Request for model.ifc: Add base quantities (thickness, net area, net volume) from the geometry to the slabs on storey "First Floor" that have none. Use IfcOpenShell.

First a look at what the model holds.

```python
import ifcopenshell
import ifcopenshell.util.element
import ifcopenshell.util.unit

model = ifcopenshell.open("model.ifc")
print(model.schema)
for unit_type in ("LENGTHUNIT", "AREAUNIT", "VOLUMEUNIT"):
    print(unit_type, ifcopenshell.util.unit.calculate_unit_scale(model, unit_type))
storey = next(s for s in model.by_type("IfcBuildingStorey") if s.Name == "First Floor")
slabs = [e for e in ifcopenshell.util.element.get_decomposition(storey) if e.is_a("IfcSlab")]
for e in sorted(slabs, key=lambda e: e.id()):
    print(e.id(), e.is_a(), e.Name, list(ifcopenshell.util.element.get_psets(e, qtos_only=True)), sep=" | ")
```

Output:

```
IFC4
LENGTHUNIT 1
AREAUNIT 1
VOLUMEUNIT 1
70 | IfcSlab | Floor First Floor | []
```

```python
import ifcopenshell
import ifcopenshell.api.pset
import ifcopenshell.geom
import ifcopenshell.util.element
import ifcopenshell.util.shape
import ifcopenshell.util.unit

model = ifcopenshell.open("model.ifc")
unit_scale = ifcopenshell.util.unit.calculate_unit_scale(model)
area_scale = ifcopenshell.util.unit.calculate_unit_scale(model, "AREAUNIT")
volume_scale = ifcopenshell.util.unit.calculate_unit_scale(model, "VOLUMEUNIT")
settings = ifcopenshell.geom.settings()

storey = next(s for s in model.by_type("IfcBuildingStorey") if s.Name == "First Floor")
slabs = [e for e in ifcopenshell.util.element.get_decomposition(storey) if e.is_a("IfcSlab")]

for e in sorted(slabs, key=lambda e: e.id()):
    if ifcopenshell.util.element.get_psets(e, qtos_only=True, should_inherit=False):
        continue
    # Geometry comes back in metres, in the element's own axes.
    shape = ifcopenshell.geom.create_shape(settings, e)
    values = {
        "Width": ifcopenshell.util.shape.get_z(shape.geometry) / unit_scale,
        "NetArea": ifcopenshell.util.shape.get_footprint_area(shape.geometry) / area_scale,
        "NetVolume": ifcopenshell.util.shape.get_volume(shape.geometry) / volume_scale,
    }
    qto = ifcopenshell.api.pset.add_qto(model, product=e, name="Qto_SlabBaseQuantities")
    ifcopenshell.api.pset.edit_qto(model, qto=qto, properties=values)
    print(e.id(), {k: round(v, 3) for k, v in values.items()})

model.write("model-out.ifc")
```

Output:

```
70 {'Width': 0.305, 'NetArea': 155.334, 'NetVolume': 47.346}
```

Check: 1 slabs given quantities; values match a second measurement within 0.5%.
